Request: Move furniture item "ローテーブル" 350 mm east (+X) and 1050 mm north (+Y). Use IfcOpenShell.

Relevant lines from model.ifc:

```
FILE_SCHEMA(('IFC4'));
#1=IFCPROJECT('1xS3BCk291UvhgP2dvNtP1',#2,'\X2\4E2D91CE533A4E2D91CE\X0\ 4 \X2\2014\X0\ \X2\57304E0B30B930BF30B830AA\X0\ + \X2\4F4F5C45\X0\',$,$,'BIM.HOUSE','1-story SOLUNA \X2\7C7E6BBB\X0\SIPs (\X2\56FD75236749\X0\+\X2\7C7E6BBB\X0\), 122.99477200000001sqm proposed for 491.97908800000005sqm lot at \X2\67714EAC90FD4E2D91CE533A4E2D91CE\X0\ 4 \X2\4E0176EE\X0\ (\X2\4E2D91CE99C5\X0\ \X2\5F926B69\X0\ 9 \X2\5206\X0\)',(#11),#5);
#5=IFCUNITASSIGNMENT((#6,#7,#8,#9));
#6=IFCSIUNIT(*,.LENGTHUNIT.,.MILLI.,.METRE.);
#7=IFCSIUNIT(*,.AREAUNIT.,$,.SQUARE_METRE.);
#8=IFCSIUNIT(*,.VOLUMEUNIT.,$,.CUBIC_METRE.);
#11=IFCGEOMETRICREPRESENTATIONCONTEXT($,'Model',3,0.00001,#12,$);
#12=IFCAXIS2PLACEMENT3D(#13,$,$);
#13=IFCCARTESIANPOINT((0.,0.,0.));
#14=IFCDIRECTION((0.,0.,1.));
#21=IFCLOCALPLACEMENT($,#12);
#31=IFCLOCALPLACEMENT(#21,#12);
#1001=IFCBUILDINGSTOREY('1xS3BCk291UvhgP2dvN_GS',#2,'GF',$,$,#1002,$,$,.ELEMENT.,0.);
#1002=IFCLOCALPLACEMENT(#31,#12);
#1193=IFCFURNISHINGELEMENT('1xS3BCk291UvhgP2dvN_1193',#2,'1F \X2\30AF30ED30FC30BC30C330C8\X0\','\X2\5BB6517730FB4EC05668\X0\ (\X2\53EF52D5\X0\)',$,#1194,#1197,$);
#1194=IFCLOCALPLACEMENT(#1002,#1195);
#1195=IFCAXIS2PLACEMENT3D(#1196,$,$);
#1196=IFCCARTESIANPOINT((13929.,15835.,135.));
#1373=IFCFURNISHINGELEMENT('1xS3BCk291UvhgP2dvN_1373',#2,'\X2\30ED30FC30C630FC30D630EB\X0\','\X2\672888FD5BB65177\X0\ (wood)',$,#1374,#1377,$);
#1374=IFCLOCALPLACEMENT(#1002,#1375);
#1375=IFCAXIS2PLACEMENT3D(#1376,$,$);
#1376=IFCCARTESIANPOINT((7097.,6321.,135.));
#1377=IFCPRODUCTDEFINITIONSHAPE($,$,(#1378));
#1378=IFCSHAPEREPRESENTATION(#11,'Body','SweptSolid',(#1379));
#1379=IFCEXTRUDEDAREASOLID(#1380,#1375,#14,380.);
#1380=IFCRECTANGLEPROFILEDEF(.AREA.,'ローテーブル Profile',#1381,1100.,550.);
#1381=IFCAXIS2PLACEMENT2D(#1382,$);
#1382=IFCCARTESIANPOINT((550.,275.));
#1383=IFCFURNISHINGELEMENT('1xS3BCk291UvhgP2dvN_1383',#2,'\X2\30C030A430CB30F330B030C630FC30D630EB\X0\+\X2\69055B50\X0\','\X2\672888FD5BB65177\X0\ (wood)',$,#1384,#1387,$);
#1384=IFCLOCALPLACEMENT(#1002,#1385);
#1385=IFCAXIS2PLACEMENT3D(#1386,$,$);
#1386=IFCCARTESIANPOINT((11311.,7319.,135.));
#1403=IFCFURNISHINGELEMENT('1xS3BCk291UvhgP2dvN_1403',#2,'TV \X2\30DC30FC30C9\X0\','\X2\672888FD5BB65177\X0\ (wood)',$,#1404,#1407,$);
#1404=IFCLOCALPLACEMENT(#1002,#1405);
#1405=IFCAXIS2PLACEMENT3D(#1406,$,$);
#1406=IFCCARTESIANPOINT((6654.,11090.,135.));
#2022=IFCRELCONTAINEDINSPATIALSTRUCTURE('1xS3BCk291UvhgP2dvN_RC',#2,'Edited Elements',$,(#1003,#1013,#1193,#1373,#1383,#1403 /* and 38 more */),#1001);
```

```python
import ifcopenshell
import ifcopenshell.api.geometry
import ifcopenshell.util.placement

model = ifcopenshell.open("model.ifc")

item = model.by_guid("1xS3BCk291UvhgP2dvN_1373")
matrix = ifcopenshell.util.placement.get_local_placement(item.ObjectPlacement)
matrix[0, 3] += 350.0
matrix[1, 3] += 1050.0
ifcopenshell.api.geometry.edit_object_placement(model, product=item, matrix=matrix, is_si=False)

print(ifcopenshell.util.placement.get_local_placement(item.ObjectPlacement).round(3) + 0.0)

model.write("model-out.ifc")
```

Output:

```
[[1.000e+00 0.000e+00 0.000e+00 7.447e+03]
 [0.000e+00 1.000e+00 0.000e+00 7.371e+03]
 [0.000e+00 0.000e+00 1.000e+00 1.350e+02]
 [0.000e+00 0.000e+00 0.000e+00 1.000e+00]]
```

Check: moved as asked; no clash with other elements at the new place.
